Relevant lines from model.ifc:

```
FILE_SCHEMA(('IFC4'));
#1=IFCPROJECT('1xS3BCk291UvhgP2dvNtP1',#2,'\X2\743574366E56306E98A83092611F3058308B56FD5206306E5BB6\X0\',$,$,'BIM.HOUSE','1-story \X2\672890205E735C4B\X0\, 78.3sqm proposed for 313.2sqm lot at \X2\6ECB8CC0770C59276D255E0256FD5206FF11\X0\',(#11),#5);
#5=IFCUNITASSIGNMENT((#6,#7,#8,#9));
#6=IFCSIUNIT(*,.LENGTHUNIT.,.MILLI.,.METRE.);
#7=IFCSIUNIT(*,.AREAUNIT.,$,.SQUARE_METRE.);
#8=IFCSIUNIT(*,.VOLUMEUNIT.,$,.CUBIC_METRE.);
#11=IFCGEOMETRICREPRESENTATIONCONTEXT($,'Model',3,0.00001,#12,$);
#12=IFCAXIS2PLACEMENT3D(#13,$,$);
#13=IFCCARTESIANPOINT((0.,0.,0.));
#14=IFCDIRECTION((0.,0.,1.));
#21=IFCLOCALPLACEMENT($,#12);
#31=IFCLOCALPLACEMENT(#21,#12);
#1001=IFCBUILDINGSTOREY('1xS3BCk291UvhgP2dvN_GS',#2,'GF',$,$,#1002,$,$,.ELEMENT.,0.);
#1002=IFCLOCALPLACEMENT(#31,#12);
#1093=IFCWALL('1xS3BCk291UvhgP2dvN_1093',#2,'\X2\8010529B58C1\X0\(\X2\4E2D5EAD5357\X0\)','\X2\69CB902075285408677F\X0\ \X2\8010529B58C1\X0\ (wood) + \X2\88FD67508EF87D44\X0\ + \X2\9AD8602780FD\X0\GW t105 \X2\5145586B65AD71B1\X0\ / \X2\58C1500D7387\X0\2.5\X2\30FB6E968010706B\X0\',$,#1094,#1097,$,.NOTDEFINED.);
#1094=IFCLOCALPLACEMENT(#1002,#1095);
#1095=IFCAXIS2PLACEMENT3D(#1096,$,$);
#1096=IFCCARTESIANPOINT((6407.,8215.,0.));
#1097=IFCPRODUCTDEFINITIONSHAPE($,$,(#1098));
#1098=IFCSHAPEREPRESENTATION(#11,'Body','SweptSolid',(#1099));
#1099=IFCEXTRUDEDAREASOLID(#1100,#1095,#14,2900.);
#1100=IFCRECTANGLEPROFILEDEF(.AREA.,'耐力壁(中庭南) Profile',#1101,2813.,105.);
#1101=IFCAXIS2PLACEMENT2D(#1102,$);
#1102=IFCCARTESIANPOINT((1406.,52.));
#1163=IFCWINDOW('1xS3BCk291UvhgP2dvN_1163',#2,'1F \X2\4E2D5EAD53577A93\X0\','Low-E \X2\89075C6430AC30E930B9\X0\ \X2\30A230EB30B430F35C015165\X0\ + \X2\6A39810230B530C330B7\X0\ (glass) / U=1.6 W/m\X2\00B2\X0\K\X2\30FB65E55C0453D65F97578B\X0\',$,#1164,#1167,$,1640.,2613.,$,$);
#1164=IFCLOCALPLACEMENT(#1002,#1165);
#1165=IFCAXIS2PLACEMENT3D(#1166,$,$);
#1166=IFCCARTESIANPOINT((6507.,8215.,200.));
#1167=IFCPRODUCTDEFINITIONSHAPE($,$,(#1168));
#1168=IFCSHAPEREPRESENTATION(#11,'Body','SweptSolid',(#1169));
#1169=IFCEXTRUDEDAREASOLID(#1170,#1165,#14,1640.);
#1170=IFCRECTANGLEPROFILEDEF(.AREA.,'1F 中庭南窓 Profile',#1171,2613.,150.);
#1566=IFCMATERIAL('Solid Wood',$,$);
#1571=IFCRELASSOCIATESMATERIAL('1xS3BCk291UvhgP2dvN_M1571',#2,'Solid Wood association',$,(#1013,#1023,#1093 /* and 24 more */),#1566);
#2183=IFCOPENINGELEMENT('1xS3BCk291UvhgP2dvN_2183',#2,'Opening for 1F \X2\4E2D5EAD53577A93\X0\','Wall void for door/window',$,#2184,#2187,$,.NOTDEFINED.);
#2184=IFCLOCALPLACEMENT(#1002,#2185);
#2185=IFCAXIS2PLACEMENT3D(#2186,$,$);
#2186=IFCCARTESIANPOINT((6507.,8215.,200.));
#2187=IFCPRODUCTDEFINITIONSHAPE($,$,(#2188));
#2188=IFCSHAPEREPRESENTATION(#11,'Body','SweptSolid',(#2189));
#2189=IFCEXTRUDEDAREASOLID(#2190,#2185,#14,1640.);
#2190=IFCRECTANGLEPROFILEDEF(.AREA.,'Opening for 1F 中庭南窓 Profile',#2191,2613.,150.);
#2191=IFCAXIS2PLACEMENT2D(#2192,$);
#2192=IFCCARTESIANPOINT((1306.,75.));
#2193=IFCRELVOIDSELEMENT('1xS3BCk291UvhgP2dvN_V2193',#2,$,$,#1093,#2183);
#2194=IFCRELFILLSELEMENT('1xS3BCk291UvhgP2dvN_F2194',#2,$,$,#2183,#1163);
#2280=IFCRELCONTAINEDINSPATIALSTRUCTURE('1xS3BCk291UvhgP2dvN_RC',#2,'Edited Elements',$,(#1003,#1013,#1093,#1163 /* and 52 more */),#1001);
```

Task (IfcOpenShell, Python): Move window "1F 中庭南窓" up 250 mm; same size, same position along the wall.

```python
import numpy as np
import ifcopenshell
import ifcopenshell.api.geometry
import ifcopenshell.util.placement
import ifcopenshell.util.unit

model = ifcopenshell.open("model.ifc")
unit_scale = ifcopenshell.util.unit.calculate_unit_scale(model)

window = model.by_guid("1xS3BCk291UvhgP2dvN_1163")
opening = window.FillsVoids[0].RelatingOpeningElement
dz = 0.25 / unit_scale

shift = np.array([0.0, 0.0, dz])
# The window is not placed relative to its opening, so move both.
for product in (opening, window):
    matrix = ifcopenshell.util.placement.get_local_placement(product.ObjectPlacement)
    matrix[:3, 3] += shift
    ifcopenshell.api.geometry.edit_object_placement(model, product=product, matrix=matrix, is_si=False)

print(f"moved by {dz * unit_scale:+.3f} m")

model.write("model-out.ifc")
```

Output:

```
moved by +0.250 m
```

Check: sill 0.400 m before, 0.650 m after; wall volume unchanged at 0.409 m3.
